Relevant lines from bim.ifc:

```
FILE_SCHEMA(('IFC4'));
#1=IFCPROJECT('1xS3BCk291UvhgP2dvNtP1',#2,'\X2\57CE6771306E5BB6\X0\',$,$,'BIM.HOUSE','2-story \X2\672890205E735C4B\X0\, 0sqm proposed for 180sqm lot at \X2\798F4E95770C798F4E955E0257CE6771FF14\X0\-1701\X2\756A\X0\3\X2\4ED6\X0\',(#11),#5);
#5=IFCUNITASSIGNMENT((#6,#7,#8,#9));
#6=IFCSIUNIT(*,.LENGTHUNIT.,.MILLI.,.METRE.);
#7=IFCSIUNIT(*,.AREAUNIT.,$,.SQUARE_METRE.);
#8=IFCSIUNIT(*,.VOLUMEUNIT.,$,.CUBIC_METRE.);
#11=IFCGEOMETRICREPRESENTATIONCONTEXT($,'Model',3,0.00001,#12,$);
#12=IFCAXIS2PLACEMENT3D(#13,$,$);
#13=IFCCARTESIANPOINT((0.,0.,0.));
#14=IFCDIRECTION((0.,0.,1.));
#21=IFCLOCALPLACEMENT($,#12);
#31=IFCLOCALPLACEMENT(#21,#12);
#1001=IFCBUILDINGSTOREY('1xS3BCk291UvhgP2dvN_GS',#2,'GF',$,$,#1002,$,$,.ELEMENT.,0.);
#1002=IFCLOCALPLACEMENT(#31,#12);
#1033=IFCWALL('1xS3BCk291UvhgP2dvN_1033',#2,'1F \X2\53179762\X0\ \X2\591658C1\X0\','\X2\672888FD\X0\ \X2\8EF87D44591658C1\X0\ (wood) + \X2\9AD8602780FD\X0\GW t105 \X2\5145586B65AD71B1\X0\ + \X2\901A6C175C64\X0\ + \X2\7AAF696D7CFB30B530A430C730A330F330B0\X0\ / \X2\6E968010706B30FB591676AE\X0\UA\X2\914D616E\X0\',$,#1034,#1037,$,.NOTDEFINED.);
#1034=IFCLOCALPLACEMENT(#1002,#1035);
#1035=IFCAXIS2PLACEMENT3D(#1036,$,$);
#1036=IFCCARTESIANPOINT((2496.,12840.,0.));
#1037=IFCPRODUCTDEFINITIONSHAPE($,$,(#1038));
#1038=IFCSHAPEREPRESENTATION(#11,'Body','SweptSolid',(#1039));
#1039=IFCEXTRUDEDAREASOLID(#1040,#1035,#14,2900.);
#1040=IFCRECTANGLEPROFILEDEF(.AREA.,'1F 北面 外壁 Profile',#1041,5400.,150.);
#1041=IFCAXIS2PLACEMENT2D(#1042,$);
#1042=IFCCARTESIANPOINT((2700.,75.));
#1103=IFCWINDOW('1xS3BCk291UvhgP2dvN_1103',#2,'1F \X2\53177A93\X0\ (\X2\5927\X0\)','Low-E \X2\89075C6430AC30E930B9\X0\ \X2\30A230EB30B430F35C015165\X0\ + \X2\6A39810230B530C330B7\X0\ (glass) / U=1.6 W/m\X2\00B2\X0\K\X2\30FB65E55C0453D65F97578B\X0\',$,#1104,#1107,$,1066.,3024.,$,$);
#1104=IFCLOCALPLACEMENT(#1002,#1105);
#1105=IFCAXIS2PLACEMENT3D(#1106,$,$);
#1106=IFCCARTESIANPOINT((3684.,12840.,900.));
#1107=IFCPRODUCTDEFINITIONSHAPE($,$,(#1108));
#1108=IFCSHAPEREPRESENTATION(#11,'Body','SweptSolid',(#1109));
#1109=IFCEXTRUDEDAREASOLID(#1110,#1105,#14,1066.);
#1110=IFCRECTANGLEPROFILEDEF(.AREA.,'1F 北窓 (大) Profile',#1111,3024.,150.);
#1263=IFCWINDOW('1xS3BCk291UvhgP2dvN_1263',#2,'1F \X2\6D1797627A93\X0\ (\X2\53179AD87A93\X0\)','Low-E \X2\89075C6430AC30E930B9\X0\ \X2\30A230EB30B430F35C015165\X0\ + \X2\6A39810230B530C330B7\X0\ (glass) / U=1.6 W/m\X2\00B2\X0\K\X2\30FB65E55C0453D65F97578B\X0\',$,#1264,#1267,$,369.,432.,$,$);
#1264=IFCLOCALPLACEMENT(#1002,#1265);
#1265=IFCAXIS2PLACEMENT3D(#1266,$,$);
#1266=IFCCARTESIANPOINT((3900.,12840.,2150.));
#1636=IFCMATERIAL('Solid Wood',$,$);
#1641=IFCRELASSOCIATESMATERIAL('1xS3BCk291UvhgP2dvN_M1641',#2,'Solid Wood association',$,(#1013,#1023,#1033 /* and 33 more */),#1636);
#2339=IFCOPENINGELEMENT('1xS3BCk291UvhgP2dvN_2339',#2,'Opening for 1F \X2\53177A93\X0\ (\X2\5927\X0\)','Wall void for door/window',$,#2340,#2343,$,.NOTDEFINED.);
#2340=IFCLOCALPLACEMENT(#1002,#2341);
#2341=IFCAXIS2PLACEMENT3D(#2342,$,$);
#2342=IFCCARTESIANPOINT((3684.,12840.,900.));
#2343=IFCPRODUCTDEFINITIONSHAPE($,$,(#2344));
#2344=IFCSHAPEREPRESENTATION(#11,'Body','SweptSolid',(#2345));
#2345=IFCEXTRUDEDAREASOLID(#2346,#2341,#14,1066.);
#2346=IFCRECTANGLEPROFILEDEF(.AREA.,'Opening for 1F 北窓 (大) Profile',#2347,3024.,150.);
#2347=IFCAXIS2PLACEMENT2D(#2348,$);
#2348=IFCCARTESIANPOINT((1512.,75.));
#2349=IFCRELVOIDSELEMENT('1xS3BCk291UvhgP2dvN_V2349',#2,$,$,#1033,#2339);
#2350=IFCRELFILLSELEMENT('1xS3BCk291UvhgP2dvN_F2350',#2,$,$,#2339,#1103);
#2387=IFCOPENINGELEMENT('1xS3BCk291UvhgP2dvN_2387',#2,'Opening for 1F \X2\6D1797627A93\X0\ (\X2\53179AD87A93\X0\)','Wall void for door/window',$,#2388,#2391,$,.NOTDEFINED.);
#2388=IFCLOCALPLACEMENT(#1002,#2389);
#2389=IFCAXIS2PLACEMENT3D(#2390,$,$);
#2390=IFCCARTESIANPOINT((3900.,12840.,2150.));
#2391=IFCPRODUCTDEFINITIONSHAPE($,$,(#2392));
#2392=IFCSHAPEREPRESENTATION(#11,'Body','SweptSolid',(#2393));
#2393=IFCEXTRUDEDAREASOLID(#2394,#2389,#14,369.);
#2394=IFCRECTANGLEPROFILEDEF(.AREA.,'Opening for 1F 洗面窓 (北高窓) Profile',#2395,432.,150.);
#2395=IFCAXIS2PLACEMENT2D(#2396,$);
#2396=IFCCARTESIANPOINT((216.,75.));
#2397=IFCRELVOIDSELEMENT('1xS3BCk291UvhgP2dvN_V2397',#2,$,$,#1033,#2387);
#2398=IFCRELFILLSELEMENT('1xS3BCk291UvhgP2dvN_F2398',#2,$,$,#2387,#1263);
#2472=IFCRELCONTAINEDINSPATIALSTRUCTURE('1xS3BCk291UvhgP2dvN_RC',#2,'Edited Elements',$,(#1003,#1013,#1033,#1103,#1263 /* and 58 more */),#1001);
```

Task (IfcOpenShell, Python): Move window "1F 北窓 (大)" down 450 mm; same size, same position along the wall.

```python
import numpy as np
import ifcopenshell
import ifcopenshell.api.geometry
import ifcopenshell.util.placement
import ifcopenshell.util.unit

model = ifcopenshell.open("bim.ifc")
unit_scale = ifcopenshell.util.unit.calculate_unit_scale(model)

window = model.by_guid("1xS3BCk291UvhgP2dvN_1103")
opening = window.FillsVoids[0].RelatingOpeningElement
dz = -450.0

shift = np.array([0.0, 0.0, dz])
# The window is not placed relative to its opening, so move both.
for product in (opening, window):
    matrix = ifcopenshell.util.placement.get_local_placement(product.ObjectPlacement)
    matrix[:3, 3] += shift
    ifcopenshell.api.geometry.edit_object_placement(model, product=product, matrix=matrix, is_si=False)

print(f"moved by {dz * unit_scale:+.3f} m")

model.write("bim_rev.ifc")
```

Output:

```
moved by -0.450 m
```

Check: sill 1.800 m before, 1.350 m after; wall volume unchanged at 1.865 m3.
